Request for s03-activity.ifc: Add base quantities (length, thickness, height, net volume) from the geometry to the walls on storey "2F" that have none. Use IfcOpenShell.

First a look at what the model holds.

```python
import ifcopenshell
import ifcopenshell.util.element
import ifcopenshell.util.unit

model = ifcopenshell.open("s03-activity.ifc")
print(model.schema)
for unit_type in ("LENGTHUNIT", "AREAUNIT", "VOLUMEUNIT"):
    print(unit_type, ifcopenshell.util.unit.calculate_unit_scale(model, unit_type))
storey = next(s for s in model.by_type("IfcBuildingStorey") if s.Name == "2F")
walls = [e for e in ifcopenshell.util.element.get_decomposition(storey) if e.is_a("IfcWall")]
for e in sorted(walls, key=lambda e: e.id()):
    print(e.id(), e.is_a(), e.Name, list(ifcopenshell.util.element.get_psets(e, qtos_only=True)), sep=" | ")
```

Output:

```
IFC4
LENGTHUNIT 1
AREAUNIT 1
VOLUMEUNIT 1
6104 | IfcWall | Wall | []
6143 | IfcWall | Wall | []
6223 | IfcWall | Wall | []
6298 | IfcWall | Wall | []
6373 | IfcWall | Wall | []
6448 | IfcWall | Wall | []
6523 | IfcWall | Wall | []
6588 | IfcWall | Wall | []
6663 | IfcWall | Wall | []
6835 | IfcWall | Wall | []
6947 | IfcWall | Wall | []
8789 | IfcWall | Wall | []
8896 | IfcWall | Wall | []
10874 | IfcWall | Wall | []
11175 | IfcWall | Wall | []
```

```python
import ifcopenshell
import ifcopenshell.api.pset
import ifcopenshell.geom
import ifcopenshell.util.element
import ifcopenshell.util.shape
import ifcopenshell.util.unit

model = ifcopenshell.open("s03-activity.ifc")
unit_scale = ifcopenshell.util.unit.calculate_unit_scale(model)
volume_scale = ifcopenshell.util.unit.calculate_unit_scale(model, "VOLUMEUNIT")
settings = ifcopenshell.geom.settings()

storey = next(s for s in model.by_type("IfcBuildingStorey") if s.Name == "2F")
walls = [e for e in ifcopenshell.util.element.get_decomposition(storey) if e.is_a("IfcWall")]

for e in sorted(walls, key=lambda e: e.id()):
    if ifcopenshell.util.element.get_psets(e, qtos_only=True, should_inherit=False):
        continue
    # Geometry comes back in metres, in the element's own axes.
    shape = ifcopenshell.geom.create_shape(settings, e)
    values = {
        "Length": ifcopenshell.util.shape.get_x(shape.geometry) / unit_scale,
        "Width": ifcopenshell.util.shape.get_y(shape.geometry) / unit_scale,
        "Height": ifcopenshell.util.shape.get_z(shape.geometry) / unit_scale,
        "NetVolume": ifcopenshell.util.shape.get_volume(shape.geometry) / volume_scale,
    }
    qto = ifcopenshell.api.pset.add_qto(model, product=e, name="Qto_WallBaseQuantities")
    ifcopenshell.api.pset.edit_qto(model, qto=qto, properties=values)
    print(e.id(), {k: round(v, 3) for k, v in values.items()})

model.write("s03-activity_edited.ifc")
```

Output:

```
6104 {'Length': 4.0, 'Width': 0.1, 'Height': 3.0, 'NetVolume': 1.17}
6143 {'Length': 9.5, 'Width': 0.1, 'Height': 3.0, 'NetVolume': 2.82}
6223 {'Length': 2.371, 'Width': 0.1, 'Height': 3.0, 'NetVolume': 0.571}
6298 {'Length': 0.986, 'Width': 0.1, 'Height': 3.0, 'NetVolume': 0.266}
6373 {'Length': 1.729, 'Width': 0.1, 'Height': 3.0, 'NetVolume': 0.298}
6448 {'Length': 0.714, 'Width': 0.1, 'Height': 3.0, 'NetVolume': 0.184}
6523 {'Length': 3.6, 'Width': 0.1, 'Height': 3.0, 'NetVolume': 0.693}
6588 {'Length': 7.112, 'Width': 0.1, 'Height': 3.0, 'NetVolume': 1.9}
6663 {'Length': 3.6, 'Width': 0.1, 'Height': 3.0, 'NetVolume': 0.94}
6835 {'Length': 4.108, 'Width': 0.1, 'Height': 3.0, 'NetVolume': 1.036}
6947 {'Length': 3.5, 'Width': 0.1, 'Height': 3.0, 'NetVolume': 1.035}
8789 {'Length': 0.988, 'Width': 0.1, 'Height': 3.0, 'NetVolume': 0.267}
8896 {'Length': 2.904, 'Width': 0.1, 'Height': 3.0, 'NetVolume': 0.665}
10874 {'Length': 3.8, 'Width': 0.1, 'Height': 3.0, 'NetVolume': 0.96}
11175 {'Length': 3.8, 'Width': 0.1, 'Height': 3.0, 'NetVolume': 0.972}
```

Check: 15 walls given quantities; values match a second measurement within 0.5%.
